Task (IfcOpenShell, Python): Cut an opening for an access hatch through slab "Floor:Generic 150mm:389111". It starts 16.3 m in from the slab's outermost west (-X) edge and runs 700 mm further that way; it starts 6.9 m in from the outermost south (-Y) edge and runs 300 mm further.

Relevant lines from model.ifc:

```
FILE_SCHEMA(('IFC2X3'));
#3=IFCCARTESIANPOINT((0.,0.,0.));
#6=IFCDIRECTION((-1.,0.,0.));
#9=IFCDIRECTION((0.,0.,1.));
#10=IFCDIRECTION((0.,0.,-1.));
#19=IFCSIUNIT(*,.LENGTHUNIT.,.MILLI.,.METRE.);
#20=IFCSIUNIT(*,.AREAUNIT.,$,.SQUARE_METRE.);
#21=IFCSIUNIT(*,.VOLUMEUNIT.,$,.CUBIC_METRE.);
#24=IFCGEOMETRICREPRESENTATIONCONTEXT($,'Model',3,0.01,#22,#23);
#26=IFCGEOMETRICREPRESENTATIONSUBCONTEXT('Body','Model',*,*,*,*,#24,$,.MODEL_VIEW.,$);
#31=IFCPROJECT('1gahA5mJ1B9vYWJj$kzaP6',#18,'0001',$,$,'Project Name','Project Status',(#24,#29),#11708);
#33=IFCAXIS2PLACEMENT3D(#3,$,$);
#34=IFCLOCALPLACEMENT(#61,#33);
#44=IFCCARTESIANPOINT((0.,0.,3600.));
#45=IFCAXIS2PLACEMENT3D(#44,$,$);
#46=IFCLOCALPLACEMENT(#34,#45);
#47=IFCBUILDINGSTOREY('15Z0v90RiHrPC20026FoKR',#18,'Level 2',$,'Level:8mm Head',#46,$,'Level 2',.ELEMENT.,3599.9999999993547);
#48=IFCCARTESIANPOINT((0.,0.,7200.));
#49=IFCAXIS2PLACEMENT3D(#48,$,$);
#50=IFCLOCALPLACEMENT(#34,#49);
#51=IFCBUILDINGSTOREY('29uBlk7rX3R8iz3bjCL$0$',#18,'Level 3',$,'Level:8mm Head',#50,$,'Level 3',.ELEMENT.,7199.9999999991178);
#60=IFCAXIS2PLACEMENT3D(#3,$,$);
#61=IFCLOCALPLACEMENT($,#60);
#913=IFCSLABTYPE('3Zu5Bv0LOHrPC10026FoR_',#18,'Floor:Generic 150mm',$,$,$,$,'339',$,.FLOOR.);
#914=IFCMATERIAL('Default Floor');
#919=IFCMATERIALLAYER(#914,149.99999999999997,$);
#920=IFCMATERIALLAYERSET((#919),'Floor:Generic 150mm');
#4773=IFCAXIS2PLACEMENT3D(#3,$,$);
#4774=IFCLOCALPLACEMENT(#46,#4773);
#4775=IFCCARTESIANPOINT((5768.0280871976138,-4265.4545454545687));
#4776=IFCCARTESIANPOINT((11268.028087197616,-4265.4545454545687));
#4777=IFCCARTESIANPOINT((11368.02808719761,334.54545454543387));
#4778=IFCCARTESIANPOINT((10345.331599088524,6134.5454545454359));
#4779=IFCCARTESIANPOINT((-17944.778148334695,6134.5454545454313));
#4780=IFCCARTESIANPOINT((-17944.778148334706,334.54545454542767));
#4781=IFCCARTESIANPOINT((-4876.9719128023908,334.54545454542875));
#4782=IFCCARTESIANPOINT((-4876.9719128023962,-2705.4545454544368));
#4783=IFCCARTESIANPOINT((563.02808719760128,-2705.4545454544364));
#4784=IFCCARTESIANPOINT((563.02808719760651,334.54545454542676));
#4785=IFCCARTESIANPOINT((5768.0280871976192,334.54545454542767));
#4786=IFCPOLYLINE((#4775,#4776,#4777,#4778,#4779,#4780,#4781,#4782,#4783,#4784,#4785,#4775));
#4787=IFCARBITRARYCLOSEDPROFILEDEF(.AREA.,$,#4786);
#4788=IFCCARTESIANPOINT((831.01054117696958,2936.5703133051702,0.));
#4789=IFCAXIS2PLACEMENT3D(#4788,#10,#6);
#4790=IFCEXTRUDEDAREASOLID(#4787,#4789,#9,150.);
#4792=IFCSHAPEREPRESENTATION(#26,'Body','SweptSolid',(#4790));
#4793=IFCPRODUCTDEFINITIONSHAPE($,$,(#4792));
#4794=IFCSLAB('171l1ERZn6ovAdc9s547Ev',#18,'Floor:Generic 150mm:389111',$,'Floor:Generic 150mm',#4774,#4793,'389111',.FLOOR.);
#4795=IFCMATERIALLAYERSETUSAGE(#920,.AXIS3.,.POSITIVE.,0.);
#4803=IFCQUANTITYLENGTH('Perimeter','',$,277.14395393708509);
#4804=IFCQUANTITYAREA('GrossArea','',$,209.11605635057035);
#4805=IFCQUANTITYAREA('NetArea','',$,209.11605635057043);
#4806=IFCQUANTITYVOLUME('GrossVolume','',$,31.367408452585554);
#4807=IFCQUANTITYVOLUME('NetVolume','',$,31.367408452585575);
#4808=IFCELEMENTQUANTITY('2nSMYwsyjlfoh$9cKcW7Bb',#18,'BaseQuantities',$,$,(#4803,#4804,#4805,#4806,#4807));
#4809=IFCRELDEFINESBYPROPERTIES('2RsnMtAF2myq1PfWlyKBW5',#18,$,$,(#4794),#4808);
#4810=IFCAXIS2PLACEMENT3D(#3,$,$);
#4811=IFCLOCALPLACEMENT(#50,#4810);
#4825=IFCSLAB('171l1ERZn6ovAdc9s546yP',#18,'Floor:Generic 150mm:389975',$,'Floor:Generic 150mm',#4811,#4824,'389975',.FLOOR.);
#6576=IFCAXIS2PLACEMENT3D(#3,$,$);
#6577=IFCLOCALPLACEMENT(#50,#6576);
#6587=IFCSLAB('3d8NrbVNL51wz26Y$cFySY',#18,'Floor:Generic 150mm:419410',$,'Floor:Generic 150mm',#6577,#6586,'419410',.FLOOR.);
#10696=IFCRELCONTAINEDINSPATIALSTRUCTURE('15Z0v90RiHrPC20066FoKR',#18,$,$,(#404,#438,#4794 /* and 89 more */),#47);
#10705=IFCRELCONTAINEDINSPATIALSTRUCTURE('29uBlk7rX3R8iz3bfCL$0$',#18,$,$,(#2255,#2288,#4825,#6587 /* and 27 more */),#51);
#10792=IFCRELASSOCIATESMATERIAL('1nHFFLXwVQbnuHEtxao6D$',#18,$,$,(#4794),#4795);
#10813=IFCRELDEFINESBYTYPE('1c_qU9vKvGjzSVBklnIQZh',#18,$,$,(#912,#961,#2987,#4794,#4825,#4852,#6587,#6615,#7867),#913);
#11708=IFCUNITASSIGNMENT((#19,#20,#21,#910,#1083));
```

```python
import numpy as np
import ifcopenshell
import ifcopenshell.api.feature
import ifcopenshell.api.geometry
import ifcopenshell.api.pset
import ifcopenshell.api.root
import ifcopenshell.geom
import ifcopenshell.util.element
import ifcopenshell.util.placement
import ifcopenshell.util.representation
import ifcopenshell.util.shape
import ifcopenshell.util.unit

model = ifcopenshell.open("model.ifc")
unit_scale = ifcopenshell.util.unit.calculate_unit_scale(model)
area_scale = ifcopenshell.util.unit.calculate_unit_scale(model, "AREAUNIT")
volume_scale = ifcopenshell.util.unit.calculate_unit_scale(model, "VOLUMEUNIT")
settings = ifcopenshell.geom.settings()


def volume(element):
    """Net volume in cubic metres, openings subtracted."""
    shape = ifcopenshell.geom.create_shape(settings, element)
    return ifcopenshell.util.shape.get_volume(shape.geometry)


slab = model.by_guid("171l1ERZn6ovAdc9s547Ev")
before = volume(slab)

# Extent in the slab's own axes, in metres. The edges named are its -X and -Y sides.
slab_shape = ifcopenshell.geom.create_shape(settings, slab)
vertices = ifcopenshell.util.shape.get_vertices(slab_shape.geometry)
x_min, y_min, bottom = vertices.min(axis=0)
top = vertices[:, 2].max()

opening = ifcopenshell.api.root.create_entity(model, ifc_class="IfcOpeningElement", name="Access hatch opening")
context = ifcopenshell.util.representation.get_context(model, "Model", "Body", "MODEL_VIEW")
width, depth = 0.7, 0.3
outline = [(0.0, 0.0), (width, 0.0), (width, depth), (0.0, depth), (0.0, 0.0)]
# Overshoot both faces by 50 mm so the cut is clean.
shape = ifcopenshell.api.geometry.add_slab_representation(
    model, context=context, depth=top - bottom + 0.1, polyline=outline
)
ifcopenshell.api.geometry.assign_representation(model, product=opening, representation=shape)

matrix = ifcopenshell.util.placement.get_local_placement(slab.ObjectPlacement)
matrix[:, 3] = matrix @ np.append(np.array([x_min + 16.3, y_min + 6.9, bottom - 0.05]) / unit_scale, 1.0)
ifcopenshell.api.geometry.edit_object_placement(model, product=opening, matrix=matrix, is_si=False)
ifcopenshell.api.feature.add_feature(model, feature=opening, element=slab)

after = volume(slab)

# Update the slab's stored quantities.
qto = model.by_id(ifcopenshell.util.element.get_pset(slab, "BaseQuantities", should_inherit=False)["id"])
ifcopenshell.api.pset.edit_qto(model, qto=qto, properties={
    "NetArea": after / (top - bottom) / area_scale,
    "NetVolume": after / volume_scale,
})

print(f"slab volume {before:.3f} -> {after:.3f} m3")

model.write("model_updated.ifc")
```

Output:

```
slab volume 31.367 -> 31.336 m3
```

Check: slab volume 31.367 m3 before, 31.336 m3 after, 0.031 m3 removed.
